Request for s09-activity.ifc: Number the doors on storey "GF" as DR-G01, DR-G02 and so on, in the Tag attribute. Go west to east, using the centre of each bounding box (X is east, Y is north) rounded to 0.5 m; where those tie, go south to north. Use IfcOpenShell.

First a look at what the model holds.

```python
import ifcopenshell
import ifcopenshell.util.element
import ifcopenshell.util.placement

model = ifcopenshell.open("s09-activity.ifc")
print(model.schema)
storey = next(s for s in model.by_type("IfcBuildingStorey") if s.Name == "GF")
doors = [e for e in ifcopenshell.util.element.get_decomposition(storey) if e.is_a("IfcDoor")]
for e in sorted(doors, key=lambda e: e.id()):
    origin = ifcopenshell.util.placement.get_local_placement(e.ObjectPlacement)[:3, 3]
    print(e.id(), e.Tag, e.Name, origin.round(2) + 0.0, sep=" | ")
```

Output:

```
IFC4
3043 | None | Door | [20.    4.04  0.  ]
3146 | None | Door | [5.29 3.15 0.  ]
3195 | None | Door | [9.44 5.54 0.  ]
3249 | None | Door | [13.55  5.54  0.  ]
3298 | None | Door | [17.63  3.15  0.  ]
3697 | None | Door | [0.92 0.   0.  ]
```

```python
import ifcopenshell
import ifcopenshell.geom
import ifcopenshell.util.element
import ifcopenshell.util.shape

model = ifcopenshell.open("s09-activity.ifc")
settings = ifcopenshell.geom.settings()
settings.set("use-world-coords", True)


def centre(element):
    shape = ifcopenshell.geom.create_shape(settings, element)
    return ifcopenshell.util.shape.get_bbox_centroid(shape.geometry)


storey = next(s for s in model.by_type("IfcBuildingStorey") if s.Name == "GF")
doors = [e for e in ifcopenshell.util.element.get_decomposition(storey) if e.is_a("IfcDoor")]

# Insertion points can sit at a corner or the storey origin, so sort by the geometry (in metres).
centres = {e: centre(e) for e in doors}
doors.sort(key=lambda e: (round(centres[e][0] / 0.5), centres[e][1]))

for i, e in enumerate(doors, start=1):
    number = f"DR-G{i:02d}"
    e.Tag = number
    print(e.id(), number)

model.write("s09-activity_edited.ifc")
```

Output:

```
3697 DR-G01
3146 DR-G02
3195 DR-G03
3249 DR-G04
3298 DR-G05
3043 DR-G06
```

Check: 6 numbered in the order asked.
